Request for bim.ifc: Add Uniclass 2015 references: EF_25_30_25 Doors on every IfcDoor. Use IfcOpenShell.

First a look at what the model holds.

```python
import ifcopenshell

model = ifcopenshell.open("bim.ifc")
print(model.schema)
print("classifications:", [c.Name for c in model.by_type("IfcClassification")])
for ifc_class in ("IfcDoor", "IfcRoof", "IfcStair", "IfcWall", "IfcWindow"):
    print(ifc_class, len(model.by_type(ifc_class)))
```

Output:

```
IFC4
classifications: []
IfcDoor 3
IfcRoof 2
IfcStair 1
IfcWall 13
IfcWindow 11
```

```python
import ifcopenshell
import ifcopenshell.api.classification

model = ifcopenshell.open("bim.ifc")

system = ifcopenshell.api.classification.add_classification(model, classification="Uniclass 2015")

codes = {
    "IfcDoor": ("EF_25_30_25", "Doors"),
}
for ifc_class, (code, name) in codes.items():
    products = model.by_type(ifc_class)
    ifcopenshell.api.classification.add_reference(
        model, products=products, classification=system, identification=code, name=name
    )
    print(code, len(products))

model.write("bim_v2.ifc")
```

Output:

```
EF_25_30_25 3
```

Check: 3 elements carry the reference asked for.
